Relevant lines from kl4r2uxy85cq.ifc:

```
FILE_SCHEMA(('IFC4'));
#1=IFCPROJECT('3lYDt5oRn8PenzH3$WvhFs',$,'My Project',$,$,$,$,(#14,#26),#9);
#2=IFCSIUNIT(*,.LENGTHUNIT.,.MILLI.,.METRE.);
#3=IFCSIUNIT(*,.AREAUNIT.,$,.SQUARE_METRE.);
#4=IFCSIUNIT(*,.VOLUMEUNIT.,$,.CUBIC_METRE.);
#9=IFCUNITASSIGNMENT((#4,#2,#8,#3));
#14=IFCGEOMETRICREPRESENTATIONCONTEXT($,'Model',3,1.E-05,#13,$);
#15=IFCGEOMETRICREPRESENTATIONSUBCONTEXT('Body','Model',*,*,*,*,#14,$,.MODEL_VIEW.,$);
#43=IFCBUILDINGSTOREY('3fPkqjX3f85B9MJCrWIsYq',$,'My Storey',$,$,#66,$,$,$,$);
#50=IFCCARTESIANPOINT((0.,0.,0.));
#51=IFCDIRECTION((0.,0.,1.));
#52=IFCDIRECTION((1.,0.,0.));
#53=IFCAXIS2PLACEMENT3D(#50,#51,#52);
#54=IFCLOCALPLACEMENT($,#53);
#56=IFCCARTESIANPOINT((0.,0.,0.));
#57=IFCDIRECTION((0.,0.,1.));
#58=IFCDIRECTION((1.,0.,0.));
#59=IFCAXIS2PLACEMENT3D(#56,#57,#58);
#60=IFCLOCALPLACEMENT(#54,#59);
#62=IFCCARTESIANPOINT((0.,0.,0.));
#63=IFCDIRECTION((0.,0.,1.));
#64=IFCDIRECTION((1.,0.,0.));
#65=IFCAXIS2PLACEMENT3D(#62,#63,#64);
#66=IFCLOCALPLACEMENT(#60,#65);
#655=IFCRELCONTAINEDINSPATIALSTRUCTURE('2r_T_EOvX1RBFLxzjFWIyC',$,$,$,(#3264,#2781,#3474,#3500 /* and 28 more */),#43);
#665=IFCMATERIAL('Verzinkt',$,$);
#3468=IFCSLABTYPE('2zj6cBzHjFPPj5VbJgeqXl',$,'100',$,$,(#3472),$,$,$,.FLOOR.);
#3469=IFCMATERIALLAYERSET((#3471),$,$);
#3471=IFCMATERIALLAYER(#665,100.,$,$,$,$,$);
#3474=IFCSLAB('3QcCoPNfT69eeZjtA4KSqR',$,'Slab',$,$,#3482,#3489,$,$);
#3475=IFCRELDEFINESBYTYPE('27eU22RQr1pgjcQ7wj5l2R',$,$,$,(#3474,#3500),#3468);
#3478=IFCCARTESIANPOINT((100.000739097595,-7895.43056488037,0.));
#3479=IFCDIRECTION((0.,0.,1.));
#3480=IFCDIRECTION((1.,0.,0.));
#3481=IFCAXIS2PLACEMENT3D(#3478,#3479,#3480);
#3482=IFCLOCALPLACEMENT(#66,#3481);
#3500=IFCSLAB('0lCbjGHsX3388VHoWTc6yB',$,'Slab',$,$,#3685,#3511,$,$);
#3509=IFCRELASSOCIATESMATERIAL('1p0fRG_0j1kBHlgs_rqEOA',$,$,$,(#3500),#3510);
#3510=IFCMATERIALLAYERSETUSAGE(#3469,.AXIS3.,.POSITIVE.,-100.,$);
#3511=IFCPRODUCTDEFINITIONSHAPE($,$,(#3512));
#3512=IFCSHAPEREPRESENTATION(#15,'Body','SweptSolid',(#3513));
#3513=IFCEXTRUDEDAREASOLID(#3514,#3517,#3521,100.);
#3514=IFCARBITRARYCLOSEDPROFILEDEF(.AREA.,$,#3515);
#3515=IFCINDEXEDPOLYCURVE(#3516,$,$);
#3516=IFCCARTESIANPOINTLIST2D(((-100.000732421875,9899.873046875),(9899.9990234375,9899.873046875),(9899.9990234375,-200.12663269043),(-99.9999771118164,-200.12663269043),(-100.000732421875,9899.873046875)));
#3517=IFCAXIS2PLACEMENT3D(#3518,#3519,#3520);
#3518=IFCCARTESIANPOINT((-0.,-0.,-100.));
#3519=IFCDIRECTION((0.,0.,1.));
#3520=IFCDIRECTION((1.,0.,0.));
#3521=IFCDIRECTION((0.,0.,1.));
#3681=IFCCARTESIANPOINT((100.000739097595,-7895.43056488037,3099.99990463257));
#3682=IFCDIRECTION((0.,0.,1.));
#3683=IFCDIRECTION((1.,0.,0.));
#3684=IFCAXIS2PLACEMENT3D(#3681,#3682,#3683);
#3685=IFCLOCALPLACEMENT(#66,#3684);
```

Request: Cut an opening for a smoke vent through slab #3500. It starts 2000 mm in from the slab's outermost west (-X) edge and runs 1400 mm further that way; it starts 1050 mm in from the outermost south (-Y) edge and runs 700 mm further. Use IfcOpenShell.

```python
import numpy as np
import ifcopenshell
import ifcopenshell.api.feature
import ifcopenshell.api.geometry
import ifcopenshell.api.root
import ifcopenshell.geom
import ifcopenshell.util.placement
import ifcopenshell.util.representation
import ifcopenshell.util.shape
import ifcopenshell.util.unit

model = ifcopenshell.open("kl4r2uxy85cq.ifc")
unit_scale = ifcopenshell.util.unit.calculate_unit_scale(model)
settings = ifcopenshell.geom.settings()


def volume(element):
    """Net volume in cubic metres, openings subtracted."""
    shape = ifcopenshell.geom.create_shape(settings, element)
    return ifcopenshell.util.shape.get_volume(shape.geometry)


slab = model.by_guid("0lCbjGHsX3388VHoWTc6yB")
before = volume(slab)

# Extent in the slab's own axes, in metres. The edges named are its -X and -Y sides.
slab_shape = ifcopenshell.geom.create_shape(settings, slab)
vertices = ifcopenshell.util.shape.get_vertices(slab_shape.geometry)
x_min, y_min, bottom = vertices.min(axis=0)
top = vertices[:, 2].max()

opening = ifcopenshell.api.root.create_entity(model, ifc_class="IfcOpeningElement", name="Smoke vent opening", predefined_type="OPENING")
context = ifcopenshell.util.representation.get_context(model, "Model", "Body", "MODEL_VIEW")
width, depth = 1.4, 0.7
outline = [(0.0, 0.0), (width, 0.0), (width, depth), (0.0, depth), (0.0, 0.0)]
# Overshoot both faces by 50 mm so the cut is clean.
shape = ifcopenshell.api.geometry.add_slab_representation(
    model, context=context, depth=top - bottom + 0.1, polyline=outline
)
ifcopenshell.api.geometry.assign_representation(model, product=opening, representation=shape)

matrix = ifcopenshell.util.placement.get_local_placement(slab.ObjectPlacement)
matrix[:, 3] = matrix @ np.append(np.array([x_min + 2, y_min + 1.05, bottom - 0.05]) / unit_scale, 1.0)
ifcopenshell.api.geometry.edit_object_placement(model, product=opening, matrix=matrix, is_si=False)
ifcopenshell.api.feature.add_feature(model, feature=opening, element=slab)

after = volume(slab)

print(f"slab volume {before:.3f} -> {after:.3f} m3")

model.write("kl4r2uxy85cq_edited.ifc")
```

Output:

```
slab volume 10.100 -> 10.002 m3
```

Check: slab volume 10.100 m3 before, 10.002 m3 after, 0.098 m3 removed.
